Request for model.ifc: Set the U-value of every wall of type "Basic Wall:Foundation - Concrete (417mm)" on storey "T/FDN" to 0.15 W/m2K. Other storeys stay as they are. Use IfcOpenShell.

First a look at what the model holds.

```python
import ifcopenshell
import ifcopenshell.util.element

model = ifcopenshell.open("model.ifc")
print(model.schema)
storey = next(s for s in model.by_type("IfcBuildingStorey") if s.Name == "T/FDN")
walls = [e for e in ifcopenshell.util.element.get_decomposition(storey) if e.is_a("IfcWall")]
seen = {}
for e in walls:
    element_type = ifcopenshell.util.element.get_type(e)
    key = (element_type.Name if element_type != e and element_type else None, ifcopenshell.util.element.get_pset(e, "Pset_WallCommon", "ThermalTransmittance"))
    seen[key] = seen.get(key, 0) + 1
for (name, value), count in sorted(seen.items(), key=str):
    print(count, "x", name, "|", value)
```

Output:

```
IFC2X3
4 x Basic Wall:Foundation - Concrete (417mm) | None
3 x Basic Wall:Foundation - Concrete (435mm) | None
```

```python
import ifcopenshell
import ifcopenshell.api.pset
import ifcopenshell.util.element

model = ifcopenshell.open("model.ifc")

storey = next(s for s in model.by_type("IfcBuildingStorey") if s.Name == "T/FDN")
walls = [e for e in ifcopenshell.util.element.get_decomposition(storey) if e.is_a("IfcWall")]

count = 0
for e in walls:
    element_type = ifcopenshell.util.element.get_type(e)
    if element_type in (None, e) or element_type.Name != "Basic Wall:Foundation - Concrete (417mm)":
        continue
    # add_pset returns the element's existing set when there is one.
    pset = ifcopenshell.api.pset.add_pset(model, product=e, name="Pset_WallCommon")
    ifcopenshell.api.pset.edit_pset(model, pset=pset, properties={"ThermalTransmittance": 0.15})
    count += 1

print(count, "walls updated")

model.write("model_updated.ifc")
```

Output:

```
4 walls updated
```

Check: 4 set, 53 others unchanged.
